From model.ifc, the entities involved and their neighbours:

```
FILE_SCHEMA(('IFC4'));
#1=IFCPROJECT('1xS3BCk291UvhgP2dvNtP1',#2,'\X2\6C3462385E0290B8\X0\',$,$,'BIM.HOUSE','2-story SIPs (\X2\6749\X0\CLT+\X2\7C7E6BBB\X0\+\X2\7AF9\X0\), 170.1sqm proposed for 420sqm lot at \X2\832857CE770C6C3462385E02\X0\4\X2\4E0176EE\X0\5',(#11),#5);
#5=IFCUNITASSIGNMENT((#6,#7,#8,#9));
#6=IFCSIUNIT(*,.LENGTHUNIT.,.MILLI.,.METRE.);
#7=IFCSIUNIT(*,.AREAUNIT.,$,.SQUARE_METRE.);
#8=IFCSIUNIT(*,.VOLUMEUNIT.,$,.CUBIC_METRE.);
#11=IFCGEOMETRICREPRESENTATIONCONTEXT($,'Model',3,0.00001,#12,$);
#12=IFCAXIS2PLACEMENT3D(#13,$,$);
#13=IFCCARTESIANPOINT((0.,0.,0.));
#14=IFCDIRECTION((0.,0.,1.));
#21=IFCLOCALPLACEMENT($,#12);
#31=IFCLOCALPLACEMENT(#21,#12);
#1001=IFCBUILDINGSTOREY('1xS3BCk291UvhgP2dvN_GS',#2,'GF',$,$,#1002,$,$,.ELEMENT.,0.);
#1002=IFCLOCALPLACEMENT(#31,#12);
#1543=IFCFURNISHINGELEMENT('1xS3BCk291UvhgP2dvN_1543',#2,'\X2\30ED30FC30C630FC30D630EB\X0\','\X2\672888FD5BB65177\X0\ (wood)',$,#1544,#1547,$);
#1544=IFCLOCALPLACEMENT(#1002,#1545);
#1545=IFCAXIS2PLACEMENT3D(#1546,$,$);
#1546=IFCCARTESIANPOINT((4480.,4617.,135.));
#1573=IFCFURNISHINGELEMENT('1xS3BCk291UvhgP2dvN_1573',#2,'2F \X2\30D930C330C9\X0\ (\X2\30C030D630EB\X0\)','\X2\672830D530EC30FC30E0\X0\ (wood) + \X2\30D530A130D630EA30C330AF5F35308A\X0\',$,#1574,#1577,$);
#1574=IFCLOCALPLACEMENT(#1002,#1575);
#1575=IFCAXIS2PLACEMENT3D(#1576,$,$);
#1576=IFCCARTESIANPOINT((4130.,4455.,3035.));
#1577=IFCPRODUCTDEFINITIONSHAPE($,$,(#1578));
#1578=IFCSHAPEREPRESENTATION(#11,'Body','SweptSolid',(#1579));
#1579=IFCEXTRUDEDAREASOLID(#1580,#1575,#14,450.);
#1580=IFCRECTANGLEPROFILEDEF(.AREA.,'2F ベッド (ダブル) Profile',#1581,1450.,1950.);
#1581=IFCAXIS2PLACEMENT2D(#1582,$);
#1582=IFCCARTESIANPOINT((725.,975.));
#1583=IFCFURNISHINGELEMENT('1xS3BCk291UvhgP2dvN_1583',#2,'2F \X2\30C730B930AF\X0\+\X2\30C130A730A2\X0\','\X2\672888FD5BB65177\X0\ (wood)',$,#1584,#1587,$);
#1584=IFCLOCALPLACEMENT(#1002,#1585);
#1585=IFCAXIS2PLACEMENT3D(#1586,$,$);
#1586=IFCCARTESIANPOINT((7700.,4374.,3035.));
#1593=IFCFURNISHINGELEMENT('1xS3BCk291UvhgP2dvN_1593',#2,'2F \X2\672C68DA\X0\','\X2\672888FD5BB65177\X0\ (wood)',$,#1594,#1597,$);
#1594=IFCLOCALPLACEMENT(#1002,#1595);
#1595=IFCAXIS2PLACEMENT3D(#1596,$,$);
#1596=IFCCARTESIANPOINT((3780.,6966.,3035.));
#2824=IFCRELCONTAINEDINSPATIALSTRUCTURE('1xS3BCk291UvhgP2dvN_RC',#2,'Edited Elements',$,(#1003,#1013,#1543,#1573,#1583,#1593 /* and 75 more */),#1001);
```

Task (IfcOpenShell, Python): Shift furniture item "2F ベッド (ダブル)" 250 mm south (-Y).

```python
import ifcopenshell
import ifcopenshell.api.geometry
import ifcopenshell.util.placement

model = ifcopenshell.open("model.ifc")

item = model.by_guid("1xS3BCk291UvhgP2dvN_1573")
matrix = ifcopenshell.util.placement.get_local_placement(item.ObjectPlacement)
matrix[1, 3] -= 250.0
ifcopenshell.api.geometry.edit_object_placement(model, product=item, matrix=matrix, is_si=False)

print(ifcopenshell.util.placement.get_local_placement(item.ObjectPlacement).round(3) + 0.0)

model.write("model_edited.ifc")
```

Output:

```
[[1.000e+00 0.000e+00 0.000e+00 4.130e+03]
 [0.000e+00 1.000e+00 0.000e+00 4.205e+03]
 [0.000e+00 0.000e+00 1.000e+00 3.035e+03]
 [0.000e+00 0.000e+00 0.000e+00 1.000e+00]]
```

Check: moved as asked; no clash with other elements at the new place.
